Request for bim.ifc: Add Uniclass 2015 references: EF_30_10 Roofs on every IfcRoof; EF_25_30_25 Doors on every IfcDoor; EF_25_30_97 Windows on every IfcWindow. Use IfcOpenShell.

First a look at what the model holds.

```python
import ifcopenshell

model = ifcopenshell.open("bim.ifc")
print(model.schema)
print("classifications:", [c.Name for c in model.by_type("IfcClassification")])
for ifc_class in ("IfcDoor", "IfcRoof", "IfcStair", "IfcWall", "IfcWindow"):
    print(ifc_class, len(model.by_type(ifc_class)))
```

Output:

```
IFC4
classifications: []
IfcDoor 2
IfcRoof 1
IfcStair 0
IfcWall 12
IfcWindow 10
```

```python
import ifcopenshell
import ifcopenshell.api.classification

model = ifcopenshell.open("bim.ifc")

system = ifcopenshell.api.classification.add_classification(model, classification="Uniclass 2015")

codes = {
    "IfcRoof": ("EF_30_10", "Roofs"),
    "IfcDoor": ("EF_25_30_25", "Doors"),
    "IfcWindow": ("EF_25_30_97", "Windows"),
}
for ifc_class, (code, name) in codes.items():
    products = model.by_type(ifc_class)
    ifcopenshell.api.classification.add_reference(
        model, products=products, classification=system, identification=code, name=name
    )
    print(code, len(products))

model.write("bim_edited.ifc")
```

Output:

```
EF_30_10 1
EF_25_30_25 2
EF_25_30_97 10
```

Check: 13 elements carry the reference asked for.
